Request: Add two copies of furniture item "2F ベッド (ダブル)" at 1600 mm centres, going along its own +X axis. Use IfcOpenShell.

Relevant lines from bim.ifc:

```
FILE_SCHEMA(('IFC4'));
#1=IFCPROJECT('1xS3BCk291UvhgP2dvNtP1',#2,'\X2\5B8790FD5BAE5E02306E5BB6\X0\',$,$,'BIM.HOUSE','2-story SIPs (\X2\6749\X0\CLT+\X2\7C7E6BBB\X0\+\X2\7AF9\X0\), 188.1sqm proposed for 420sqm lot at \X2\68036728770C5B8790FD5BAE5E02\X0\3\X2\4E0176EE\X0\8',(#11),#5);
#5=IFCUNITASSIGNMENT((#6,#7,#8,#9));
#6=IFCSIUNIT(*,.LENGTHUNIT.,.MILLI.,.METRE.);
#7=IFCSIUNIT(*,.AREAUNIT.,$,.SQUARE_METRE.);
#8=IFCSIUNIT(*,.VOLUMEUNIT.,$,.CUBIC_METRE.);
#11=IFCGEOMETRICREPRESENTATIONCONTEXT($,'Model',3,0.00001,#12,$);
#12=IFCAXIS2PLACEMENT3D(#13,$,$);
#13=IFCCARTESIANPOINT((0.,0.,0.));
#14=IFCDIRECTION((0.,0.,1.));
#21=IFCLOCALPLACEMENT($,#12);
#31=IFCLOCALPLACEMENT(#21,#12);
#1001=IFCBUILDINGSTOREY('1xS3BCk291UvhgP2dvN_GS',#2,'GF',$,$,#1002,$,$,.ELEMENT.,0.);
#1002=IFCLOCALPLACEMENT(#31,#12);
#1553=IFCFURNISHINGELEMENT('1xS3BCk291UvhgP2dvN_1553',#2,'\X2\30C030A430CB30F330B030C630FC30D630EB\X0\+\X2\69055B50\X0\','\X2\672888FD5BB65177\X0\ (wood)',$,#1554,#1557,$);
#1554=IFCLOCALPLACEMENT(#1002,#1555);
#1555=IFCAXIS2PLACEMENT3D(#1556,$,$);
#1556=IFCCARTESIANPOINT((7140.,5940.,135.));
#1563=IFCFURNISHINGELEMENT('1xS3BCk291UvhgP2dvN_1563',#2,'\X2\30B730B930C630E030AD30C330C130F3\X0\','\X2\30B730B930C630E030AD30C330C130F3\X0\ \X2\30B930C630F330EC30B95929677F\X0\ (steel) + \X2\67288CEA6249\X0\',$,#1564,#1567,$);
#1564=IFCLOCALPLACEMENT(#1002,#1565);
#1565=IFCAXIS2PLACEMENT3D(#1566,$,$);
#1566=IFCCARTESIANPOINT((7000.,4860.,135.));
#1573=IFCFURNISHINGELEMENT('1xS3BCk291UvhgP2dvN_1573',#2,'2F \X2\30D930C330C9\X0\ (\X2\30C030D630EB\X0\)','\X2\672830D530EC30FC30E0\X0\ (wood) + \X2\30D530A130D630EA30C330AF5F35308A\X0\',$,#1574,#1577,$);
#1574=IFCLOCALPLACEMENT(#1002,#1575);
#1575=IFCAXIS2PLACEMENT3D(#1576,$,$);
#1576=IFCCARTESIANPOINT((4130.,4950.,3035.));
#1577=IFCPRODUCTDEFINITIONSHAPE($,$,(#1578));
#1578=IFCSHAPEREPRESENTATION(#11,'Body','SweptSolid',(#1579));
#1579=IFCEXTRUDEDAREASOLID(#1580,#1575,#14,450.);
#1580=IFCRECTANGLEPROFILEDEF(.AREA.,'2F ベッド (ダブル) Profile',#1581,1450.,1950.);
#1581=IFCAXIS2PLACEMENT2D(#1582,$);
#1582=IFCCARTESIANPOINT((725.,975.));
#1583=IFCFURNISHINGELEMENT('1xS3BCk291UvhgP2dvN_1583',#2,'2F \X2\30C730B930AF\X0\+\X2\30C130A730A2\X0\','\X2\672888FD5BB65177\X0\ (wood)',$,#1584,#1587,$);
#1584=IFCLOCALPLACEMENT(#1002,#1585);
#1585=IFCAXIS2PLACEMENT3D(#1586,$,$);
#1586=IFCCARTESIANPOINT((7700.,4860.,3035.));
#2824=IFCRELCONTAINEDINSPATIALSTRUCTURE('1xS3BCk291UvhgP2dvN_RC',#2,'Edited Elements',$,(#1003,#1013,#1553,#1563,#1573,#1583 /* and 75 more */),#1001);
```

```python
import ifcopenshell
import ifcopenshell.api.geometry
import ifcopenshell.api.root
import ifcopenshell.util.element
import ifcopenshell.util.placement
import ifcopenshell.util.unit

model = ifcopenshell.open("bim.ifc")
unit_scale = ifcopenshell.util.unit.calculate_unit_scale(model)


def reuse_history(source, copy):
    """copy_class also copies each property set's owner history, people and application; keep the originals."""
    for rel in copy.IsDefinedBy:
        if rel.is_a("IfcRelDefinesByProperties") and (history := rel.RelatingPropertyDefinition.OwnerHistory):
            rel.RelatingPropertyDefinition.OwnerHistory = source.OwnerHistory
            ifcopenshell.util.element.remove_deep2(model, history)


source = model.by_guid("1xS3BCk291UvhgP2dvN_1573")
base = ifcopenshell.util.placement.get_local_placement(source.ObjectPlacement)
step = base[:3, 0] * 1.6 / unit_scale

for i in range(1, 3):
    copy = ifcopenshell.api.root.copy_class(model, product=source)
    copy.Representation = ifcopenshell.util.element.copy_deep(
        model, source.Representation, exclude=["IfcGeometricRepresentationContext", "IfcRepresentationMap"]
    )
    reuse_history(source, copy)
    matrix = base.copy()
    matrix[:3, 3] += i * step
    print("added at", matrix[:3, 3].round(3) + 0.0)
    ifcopenshell.api.geometry.edit_object_placement(model, product=copy, matrix=matrix, is_si=False)

model.write("bim_updated.ifc")
```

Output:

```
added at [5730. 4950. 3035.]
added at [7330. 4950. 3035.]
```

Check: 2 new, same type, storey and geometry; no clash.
